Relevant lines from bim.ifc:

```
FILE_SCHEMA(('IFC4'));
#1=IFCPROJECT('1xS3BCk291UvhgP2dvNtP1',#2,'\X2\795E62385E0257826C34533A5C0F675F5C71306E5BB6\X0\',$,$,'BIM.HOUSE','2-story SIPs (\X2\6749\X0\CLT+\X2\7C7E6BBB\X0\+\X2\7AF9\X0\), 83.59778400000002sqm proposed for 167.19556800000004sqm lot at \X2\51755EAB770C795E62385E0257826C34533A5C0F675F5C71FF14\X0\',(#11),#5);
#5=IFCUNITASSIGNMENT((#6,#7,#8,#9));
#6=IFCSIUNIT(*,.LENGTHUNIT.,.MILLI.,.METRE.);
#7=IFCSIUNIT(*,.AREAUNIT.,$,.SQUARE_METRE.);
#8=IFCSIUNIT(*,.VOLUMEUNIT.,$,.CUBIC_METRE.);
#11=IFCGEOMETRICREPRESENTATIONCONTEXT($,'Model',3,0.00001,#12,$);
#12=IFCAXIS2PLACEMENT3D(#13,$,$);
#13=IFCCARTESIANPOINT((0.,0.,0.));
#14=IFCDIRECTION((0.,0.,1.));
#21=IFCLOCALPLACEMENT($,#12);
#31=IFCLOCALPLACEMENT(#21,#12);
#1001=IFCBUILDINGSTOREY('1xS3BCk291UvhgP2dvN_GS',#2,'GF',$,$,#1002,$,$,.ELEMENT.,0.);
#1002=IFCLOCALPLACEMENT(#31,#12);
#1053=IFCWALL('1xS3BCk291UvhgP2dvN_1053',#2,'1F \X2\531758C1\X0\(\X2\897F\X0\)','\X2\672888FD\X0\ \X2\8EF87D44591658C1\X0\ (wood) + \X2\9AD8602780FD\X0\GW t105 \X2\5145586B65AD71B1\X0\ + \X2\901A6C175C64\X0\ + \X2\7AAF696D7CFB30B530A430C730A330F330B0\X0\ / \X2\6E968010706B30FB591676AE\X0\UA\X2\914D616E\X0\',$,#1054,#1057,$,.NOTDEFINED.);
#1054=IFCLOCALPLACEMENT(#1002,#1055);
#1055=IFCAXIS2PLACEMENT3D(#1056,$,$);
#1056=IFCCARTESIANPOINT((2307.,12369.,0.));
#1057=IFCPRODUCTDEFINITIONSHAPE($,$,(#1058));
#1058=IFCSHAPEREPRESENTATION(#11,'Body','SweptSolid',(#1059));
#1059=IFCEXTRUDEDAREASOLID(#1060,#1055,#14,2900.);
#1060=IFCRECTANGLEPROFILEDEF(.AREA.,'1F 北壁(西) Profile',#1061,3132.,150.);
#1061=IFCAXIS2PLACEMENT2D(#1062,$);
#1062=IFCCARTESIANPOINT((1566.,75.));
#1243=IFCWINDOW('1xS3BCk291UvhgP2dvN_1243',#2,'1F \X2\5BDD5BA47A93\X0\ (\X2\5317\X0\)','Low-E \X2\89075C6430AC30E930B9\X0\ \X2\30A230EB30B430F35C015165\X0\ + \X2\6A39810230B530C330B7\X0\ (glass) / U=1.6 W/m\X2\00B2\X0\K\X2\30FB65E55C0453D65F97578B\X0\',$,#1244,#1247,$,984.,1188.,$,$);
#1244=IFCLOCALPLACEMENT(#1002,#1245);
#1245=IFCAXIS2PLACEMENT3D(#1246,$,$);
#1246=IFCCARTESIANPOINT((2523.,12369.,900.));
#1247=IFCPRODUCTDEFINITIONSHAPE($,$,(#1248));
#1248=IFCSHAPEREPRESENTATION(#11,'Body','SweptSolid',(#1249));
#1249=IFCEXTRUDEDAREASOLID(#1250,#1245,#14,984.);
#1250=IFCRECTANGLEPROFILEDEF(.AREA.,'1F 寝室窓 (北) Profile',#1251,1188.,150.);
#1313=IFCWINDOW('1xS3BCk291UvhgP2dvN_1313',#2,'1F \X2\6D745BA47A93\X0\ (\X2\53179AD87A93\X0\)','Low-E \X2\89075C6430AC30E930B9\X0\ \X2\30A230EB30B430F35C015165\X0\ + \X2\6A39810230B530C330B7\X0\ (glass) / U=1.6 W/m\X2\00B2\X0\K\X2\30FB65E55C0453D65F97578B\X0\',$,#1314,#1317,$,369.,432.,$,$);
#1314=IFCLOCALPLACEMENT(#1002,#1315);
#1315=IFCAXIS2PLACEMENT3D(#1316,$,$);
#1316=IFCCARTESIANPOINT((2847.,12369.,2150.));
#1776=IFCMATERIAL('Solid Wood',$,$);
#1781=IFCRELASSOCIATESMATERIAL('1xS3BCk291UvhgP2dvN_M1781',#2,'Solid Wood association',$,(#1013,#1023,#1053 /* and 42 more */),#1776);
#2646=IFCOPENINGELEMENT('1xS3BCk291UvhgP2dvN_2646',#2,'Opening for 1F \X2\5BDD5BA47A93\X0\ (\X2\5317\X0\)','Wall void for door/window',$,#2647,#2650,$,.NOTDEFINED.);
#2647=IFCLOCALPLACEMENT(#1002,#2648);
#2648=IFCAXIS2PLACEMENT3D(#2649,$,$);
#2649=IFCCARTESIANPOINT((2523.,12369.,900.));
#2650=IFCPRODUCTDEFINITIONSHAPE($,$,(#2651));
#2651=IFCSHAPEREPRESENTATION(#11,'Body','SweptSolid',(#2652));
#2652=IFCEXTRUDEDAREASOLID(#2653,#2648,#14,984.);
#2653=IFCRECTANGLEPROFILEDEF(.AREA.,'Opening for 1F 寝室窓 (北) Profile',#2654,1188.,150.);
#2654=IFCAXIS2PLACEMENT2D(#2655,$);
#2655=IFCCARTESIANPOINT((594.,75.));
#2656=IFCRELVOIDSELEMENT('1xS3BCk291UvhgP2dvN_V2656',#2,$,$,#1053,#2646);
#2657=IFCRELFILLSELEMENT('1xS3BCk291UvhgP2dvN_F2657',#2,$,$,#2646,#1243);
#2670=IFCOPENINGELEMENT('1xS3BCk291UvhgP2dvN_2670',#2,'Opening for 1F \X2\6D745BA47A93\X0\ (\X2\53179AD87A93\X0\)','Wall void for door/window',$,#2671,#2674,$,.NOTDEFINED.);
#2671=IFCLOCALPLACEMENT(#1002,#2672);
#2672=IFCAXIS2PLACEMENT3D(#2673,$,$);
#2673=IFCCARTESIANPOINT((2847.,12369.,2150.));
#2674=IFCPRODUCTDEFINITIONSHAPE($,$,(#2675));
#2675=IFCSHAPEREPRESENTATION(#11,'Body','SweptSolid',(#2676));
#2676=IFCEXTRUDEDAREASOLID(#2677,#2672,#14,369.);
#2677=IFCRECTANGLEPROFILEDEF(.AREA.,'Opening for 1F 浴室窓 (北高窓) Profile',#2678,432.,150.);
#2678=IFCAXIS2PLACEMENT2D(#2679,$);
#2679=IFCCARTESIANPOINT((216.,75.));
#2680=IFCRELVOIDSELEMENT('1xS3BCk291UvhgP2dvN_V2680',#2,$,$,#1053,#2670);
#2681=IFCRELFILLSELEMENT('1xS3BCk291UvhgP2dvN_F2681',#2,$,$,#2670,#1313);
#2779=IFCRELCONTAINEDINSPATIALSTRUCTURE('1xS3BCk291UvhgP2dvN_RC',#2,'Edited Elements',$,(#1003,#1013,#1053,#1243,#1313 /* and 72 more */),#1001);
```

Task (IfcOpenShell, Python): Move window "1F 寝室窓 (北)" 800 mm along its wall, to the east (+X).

```python
import ifcopenshell
import ifcopenshell.api.geometry
import ifcopenshell.util.placement
import ifcopenshell.util.unit

model = ifcopenshell.open("bim.ifc")
unit_scale = ifcopenshell.util.unit.calculate_unit_scale(model)

window = model.by_guid("1xS3BCk291UvhgP2dvN_1243")
opening = window.FillsVoids[0].RelatingOpeningElement
wall = opening.VoidsElements[0].RelatingBuildingElement

wall_matrix = ifcopenshell.util.placement.get_local_placement(wall.ObjectPlacement)
shift = wall_matrix[:3, 0] * 0.8 / unit_scale
before = ifcopenshell.util.placement.get_local_placement(window.ObjectPlacement)[:3, 3].copy()

# The window is not placed relative to its opening, so move both.
for product in (opening, window):
    matrix = ifcopenshell.util.placement.get_local_placement(product.ObjectPlacement)
    matrix[:3, 3] += shift
    ifcopenshell.api.geometry.edit_object_placement(model, product=product, matrix=matrix, is_si=False)

after = ifcopenshell.util.placement.get_local_placement(window.ObjectPlacement)[:3, 3]
print("window moved by", (after - before).round(3) + 0.0)

model.write("bim-out.ifc")
```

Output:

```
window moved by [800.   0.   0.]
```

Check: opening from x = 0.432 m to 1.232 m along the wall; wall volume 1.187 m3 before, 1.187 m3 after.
